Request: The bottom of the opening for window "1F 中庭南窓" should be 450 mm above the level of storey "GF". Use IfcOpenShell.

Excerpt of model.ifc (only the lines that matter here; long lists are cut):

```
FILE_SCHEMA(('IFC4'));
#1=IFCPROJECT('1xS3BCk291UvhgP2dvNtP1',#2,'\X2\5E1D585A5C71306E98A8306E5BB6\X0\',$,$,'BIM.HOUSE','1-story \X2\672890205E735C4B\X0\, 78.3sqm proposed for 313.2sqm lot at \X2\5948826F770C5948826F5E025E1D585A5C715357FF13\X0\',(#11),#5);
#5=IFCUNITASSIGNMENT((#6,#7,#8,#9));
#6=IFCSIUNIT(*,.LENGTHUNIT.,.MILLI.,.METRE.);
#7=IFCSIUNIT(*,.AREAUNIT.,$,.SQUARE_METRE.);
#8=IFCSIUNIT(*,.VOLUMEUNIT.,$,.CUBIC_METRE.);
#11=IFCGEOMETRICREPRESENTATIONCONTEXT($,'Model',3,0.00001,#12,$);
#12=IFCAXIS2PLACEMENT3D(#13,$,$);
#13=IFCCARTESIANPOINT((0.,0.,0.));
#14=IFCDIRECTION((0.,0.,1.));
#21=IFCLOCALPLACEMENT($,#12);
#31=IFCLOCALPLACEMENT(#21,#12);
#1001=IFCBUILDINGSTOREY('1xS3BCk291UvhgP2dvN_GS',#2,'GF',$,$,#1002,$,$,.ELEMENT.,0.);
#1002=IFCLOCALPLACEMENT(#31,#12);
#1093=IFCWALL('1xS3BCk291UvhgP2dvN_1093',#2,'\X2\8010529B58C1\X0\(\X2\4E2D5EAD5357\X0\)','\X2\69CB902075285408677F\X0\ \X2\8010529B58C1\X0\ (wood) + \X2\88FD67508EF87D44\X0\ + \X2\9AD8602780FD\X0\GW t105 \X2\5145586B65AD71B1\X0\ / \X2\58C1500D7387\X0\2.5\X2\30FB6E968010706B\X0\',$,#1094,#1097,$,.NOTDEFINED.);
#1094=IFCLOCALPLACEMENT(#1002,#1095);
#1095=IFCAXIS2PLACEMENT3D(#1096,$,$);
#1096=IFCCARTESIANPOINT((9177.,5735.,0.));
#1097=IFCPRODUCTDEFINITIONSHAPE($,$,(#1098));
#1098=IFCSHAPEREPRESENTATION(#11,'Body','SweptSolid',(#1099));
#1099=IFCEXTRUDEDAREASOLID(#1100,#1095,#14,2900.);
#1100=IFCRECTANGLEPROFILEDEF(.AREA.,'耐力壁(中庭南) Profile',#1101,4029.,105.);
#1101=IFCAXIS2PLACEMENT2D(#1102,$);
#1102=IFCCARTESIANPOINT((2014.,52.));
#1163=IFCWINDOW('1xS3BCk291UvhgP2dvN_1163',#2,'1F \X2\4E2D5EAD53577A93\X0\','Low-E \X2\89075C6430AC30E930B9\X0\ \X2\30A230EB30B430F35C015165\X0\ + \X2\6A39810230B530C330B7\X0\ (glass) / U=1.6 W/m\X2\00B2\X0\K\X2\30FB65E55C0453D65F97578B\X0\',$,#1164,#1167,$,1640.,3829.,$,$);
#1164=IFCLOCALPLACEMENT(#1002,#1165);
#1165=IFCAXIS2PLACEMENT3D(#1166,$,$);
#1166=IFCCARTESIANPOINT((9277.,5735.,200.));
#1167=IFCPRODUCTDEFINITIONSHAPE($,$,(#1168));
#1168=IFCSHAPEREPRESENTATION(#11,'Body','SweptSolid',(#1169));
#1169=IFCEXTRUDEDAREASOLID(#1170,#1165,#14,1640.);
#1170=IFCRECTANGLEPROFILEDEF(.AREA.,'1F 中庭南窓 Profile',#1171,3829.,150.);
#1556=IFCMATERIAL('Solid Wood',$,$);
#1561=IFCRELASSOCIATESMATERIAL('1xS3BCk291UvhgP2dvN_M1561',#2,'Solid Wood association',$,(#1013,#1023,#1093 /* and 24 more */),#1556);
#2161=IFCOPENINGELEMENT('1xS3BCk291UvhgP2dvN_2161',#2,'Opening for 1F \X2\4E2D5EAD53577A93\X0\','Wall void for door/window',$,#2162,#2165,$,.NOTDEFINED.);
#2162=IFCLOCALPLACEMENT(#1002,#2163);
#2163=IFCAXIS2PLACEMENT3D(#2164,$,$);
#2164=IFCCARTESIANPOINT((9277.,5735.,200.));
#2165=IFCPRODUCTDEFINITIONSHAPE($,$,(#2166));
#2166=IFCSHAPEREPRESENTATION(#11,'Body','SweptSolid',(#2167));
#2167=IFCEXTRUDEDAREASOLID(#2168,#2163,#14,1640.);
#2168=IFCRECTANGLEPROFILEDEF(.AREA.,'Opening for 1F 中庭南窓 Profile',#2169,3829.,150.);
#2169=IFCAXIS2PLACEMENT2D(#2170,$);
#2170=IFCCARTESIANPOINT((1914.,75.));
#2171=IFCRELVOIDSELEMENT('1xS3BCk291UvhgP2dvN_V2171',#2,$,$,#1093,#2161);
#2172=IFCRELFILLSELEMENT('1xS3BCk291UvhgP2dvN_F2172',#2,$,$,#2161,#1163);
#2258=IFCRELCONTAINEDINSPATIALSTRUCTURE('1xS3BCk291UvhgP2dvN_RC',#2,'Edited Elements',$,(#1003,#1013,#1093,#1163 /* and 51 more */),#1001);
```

```python
import numpy as np
import ifcopenshell
import ifcopenshell.api.geometry
import ifcopenshell.geom
import ifcopenshell.util.element
import ifcopenshell.util.placement
import ifcopenshell.util.shape
import ifcopenshell.util.unit

model = ifcopenshell.open("model.ifc")
unit_scale = ifcopenshell.util.unit.calculate_unit_scale(model)

window = model.by_guid("1xS3BCk291UvhgP2dvN_1163")
opening = window.FillsVoids[0].RelatingOpeningElement
storey = ifcopenshell.util.element.get_container(window, ifc_class="IfcBuildingStorey")
level = ifcopenshell.util.placement.get_local_placement(storey.ObjectPlacement)[2, 3]

# The opening's origin need not be at the sill, so measure its lowest point.
shape = ifcopenshell.geom.create_shape(ifcopenshell.geom.settings(), opening)
bottom = ifcopenshell.util.shape.get_shape_bottom_elevation(shape, shape.geometry) / unit_scale
dz = level + 0.45 / unit_scale - bottom

shift = np.array([0.0, 0.0, dz])
# The window is not placed relative to its opening, so move both.
for product in (opening, window):
    matrix = ifcopenshell.util.placement.get_local_placement(product.ObjectPlacement)
    matrix[:3, 3] += shift
    ifcopenshell.api.geometry.edit_object_placement(model, product=product, matrix=matrix, is_si=False)

print(f"moved by {dz * unit_scale:+.3f} m")

model.write("model_edited.ifc")
```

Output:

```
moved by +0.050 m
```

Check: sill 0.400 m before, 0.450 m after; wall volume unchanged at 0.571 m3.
